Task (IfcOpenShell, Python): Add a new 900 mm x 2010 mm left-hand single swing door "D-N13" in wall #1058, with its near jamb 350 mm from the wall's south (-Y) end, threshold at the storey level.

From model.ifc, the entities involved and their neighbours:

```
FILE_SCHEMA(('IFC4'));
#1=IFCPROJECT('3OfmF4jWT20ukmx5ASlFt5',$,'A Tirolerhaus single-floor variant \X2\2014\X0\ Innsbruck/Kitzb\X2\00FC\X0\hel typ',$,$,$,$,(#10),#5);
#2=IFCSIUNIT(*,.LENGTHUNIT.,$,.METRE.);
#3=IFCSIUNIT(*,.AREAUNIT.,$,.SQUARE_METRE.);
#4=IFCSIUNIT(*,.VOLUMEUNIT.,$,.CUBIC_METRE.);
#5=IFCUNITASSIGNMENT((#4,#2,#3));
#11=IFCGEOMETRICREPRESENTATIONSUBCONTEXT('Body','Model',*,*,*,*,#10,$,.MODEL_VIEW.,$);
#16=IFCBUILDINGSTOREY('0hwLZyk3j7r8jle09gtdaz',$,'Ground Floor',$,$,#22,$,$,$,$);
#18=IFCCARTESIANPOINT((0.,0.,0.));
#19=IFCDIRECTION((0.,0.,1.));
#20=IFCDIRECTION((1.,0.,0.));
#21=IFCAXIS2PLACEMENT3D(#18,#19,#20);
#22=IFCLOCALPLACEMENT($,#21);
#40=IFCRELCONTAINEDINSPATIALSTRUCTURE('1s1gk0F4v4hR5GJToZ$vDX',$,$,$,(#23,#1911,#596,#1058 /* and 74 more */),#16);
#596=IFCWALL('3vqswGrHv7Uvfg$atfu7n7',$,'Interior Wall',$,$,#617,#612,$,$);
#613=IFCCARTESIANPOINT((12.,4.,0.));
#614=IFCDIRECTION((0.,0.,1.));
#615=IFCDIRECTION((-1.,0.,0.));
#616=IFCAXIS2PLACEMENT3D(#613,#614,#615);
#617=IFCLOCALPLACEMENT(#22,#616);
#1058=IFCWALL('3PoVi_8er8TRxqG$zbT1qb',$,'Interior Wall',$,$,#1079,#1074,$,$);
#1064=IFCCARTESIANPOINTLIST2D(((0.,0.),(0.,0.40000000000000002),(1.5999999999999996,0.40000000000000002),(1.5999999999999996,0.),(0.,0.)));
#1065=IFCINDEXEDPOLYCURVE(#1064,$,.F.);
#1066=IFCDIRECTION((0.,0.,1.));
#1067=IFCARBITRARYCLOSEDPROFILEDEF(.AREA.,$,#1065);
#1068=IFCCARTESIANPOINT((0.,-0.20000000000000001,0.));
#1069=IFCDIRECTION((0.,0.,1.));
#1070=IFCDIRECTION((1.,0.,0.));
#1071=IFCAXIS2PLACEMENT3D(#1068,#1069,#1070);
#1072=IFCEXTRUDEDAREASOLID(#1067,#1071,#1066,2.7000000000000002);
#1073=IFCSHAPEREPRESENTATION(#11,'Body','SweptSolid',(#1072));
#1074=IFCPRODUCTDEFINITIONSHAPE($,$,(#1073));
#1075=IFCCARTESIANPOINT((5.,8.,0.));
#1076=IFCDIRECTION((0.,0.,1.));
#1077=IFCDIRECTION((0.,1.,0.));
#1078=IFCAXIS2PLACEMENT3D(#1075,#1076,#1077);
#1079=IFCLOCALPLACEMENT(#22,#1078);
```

```python
import numpy as np
import ifcopenshell
import ifcopenshell.api.feature
import ifcopenshell.api.geometry
import ifcopenshell.api.root
import ifcopenshell.api.spatial
import ifcopenshell.geom
import ifcopenshell.util.element
import ifcopenshell.util.placement
import ifcopenshell.util.representation
import ifcopenshell.util.shape
import ifcopenshell.util.unit

model = ifcopenshell.open("model.ifc")
unit_scale = ifcopenshell.util.unit.calculate_unit_scale(model)
settings = ifcopenshell.geom.settings()


def volume(element):
    """Net volume in cubic metres, openings subtracted."""
    shape = ifcopenshell.geom.create_shape(settings, element)
    return ifcopenshell.util.shape.get_volume(shape.geometry)


wall = model.by_guid("3PoVi_8er8TRxqG$zbT1qb")
storey = ifcopenshell.util.element.get_container(wall, ifc_class="IfcBuildingStorey")
context = ifcopenshell.util.representation.get_context(model, "Model", "Body", "MODEL_VIEW")
before = volume(wall)

width, height, from_end, sill = 0.9, 2.01, 0.35, 0.0  # metres

# The wall runs along its own X axis, and the end named is its -X end.
wall_shape = ifcopenshell.geom.create_shape(settings, wall)
x, y, z = ifcopenshell.util.shape.get_vertices(wall_shape.geometry).T
start = x.min() + from_end
face, thickness = float(y.min()), float(y.max() - y.min())
wall_matrix = ifcopenshell.util.placement.get_local_placement(wall.ObjectPlacement)
level = ifcopenshell.util.placement.get_local_placement(storey.ObjectPlacement)[2, 3]


def in_wall(x, y):
    """Placement at x, y metres in the wall's axes, at sill height."""
    matrix = wall_matrix.copy()
    matrix[:, 3] = wall_matrix @ np.array([x / unit_scale, y / unit_scale, 0.0, 1.0])
    matrix[2, 3] = level + sill / unit_scale
    return matrix


# Opening: a box that overshoots both wall faces by 50 mm.
opening = ifcopenshell.api.root.create_entity(model, ifc_class="IfcOpeningElement", predefined_type="OPENING")
box = ifcopenshell.api.geometry.add_wall_representation(
    model, context=context, length=width, height=height, thickness=thickness + 0.1
)
ifcopenshell.api.geometry.assign_representation(model, product=opening, representation=box)
ifcopenshell.api.geometry.edit_object_placement(model, product=opening, matrix=in_wall(start, face - 0.05), is_si=False)
ifcopenshell.api.feature.add_feature(model, feature=opening, element=wall)

door = ifcopenshell.api.root.create_entity(model, ifc_class="IfcDoor", name="D-N13", predefined_type="DOOR")
door.OverallWidth, door.OverallHeight = width / unit_scale, height / unit_scale
door.OperationType = "SINGLE_SWING_LEFT"
body = ifcopenshell.api.geometry.add_door_representation(
    model,
    context=context,
    overall_width=door.OverallWidth,
    overall_height=door.OverallHeight,
    operation_type="SINGLE_SWING_LEFT",
    lining_properties={"LiningDepth": thickness / unit_scale, "ThresholdDepth": thickness / unit_scale},
)
ifcopenshell.api.geometry.assign_representation(model, product=door, representation=body)
ifcopenshell.api.spatial.assign_container(model, products=[door], relating_structure=storey)
ifcopenshell.api.feature.add_filling(model, opening=opening, element=door)

# The lining spans the wall, so the door starts at the wall face.
ifcopenshell.api.geometry.edit_object_placement(model, product=door, matrix=in_wall(start, face), is_si=False)

after = volume(wall)

print(f"wall volume {before:.3f} -> {after:.3f} m3")

model.write("model_rev.ifc")
```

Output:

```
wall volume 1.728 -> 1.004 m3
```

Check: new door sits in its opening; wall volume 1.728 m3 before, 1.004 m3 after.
